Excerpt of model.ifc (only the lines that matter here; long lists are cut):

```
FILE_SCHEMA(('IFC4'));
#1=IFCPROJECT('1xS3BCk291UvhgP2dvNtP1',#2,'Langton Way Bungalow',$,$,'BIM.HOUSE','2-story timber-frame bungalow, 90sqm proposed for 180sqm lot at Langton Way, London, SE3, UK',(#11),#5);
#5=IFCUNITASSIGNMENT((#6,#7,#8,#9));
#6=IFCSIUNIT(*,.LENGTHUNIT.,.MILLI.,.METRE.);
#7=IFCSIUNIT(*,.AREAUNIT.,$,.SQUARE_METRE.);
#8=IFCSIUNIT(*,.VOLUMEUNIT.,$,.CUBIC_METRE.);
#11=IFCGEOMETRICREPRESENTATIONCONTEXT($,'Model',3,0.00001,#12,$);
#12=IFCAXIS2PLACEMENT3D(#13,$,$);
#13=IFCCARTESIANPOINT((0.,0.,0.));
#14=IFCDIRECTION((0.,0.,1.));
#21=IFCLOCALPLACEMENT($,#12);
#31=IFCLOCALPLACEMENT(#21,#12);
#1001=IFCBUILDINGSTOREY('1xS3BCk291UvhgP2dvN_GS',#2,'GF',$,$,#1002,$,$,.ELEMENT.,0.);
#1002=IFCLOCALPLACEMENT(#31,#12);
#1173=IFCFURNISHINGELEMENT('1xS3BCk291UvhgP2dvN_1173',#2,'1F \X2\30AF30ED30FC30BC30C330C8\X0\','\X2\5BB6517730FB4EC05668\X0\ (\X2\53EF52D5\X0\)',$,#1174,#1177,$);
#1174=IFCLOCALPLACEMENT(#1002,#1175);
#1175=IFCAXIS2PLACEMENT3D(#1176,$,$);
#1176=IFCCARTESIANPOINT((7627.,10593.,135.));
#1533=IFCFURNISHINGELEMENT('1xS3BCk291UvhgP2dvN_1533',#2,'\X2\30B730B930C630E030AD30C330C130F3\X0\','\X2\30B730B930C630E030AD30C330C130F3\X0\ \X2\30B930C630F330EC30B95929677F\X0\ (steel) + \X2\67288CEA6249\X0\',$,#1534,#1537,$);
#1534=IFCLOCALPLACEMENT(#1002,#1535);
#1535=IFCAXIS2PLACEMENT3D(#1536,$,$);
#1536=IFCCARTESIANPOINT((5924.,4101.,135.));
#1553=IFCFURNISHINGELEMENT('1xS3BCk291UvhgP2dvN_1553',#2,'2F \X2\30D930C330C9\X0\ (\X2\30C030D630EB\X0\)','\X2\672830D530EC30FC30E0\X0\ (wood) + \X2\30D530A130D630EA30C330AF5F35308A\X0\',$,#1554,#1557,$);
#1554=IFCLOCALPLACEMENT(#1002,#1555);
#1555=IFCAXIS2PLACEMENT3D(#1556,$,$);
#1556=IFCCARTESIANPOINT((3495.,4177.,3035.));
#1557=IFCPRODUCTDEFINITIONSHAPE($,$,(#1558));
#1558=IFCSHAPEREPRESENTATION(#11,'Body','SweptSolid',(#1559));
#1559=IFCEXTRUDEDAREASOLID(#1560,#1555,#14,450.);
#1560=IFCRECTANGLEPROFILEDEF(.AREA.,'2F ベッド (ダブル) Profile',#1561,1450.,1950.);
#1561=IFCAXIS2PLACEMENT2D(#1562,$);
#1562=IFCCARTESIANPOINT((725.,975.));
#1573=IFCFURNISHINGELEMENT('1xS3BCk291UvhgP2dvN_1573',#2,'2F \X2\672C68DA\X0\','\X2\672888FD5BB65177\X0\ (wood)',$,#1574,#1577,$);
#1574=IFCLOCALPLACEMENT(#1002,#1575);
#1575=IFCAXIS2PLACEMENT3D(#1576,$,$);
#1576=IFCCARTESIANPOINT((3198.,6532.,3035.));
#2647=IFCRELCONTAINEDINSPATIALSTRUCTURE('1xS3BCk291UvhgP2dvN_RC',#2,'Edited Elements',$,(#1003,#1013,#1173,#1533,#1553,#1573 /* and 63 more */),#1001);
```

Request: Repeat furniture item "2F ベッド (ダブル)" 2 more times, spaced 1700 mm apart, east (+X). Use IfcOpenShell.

```python
import numpy as np
import ifcopenshell
import ifcopenshell.api.geometry
import ifcopenshell.api.root
import ifcopenshell.util.element
import ifcopenshell.util.placement
import ifcopenshell.util.unit

model = ifcopenshell.open("model.ifc")
unit_scale = ifcopenshell.util.unit.calculate_unit_scale(model)


def reuse_history(source, copy):
    """copy_class also copies each property set's owner history, people and application; keep the originals."""
    for rel in copy.IsDefinedBy:
        if rel.is_a("IfcRelDefinesByProperties") and (history := rel.RelatingPropertyDefinition.OwnerHistory):
            rel.RelatingPropertyDefinition.OwnerHistory = source.OwnerHistory
            ifcopenshell.util.element.remove_deep2(model, history)


source = model.by_id(1553)
base = ifcopenshell.util.placement.get_local_placement(source.ObjectPlacement)
step = np.array([1.0, 0.0, 0.0]) * 1.7 / unit_scale

for i in range(1, 3):
    copy = ifcopenshell.api.root.copy_class(model, product=source)
    copy.Representation = ifcopenshell.util.element.copy_deep(
        model, source.Representation, exclude=["IfcGeometricRepresentationContext", "IfcRepresentationMap"]
    )
    reuse_history(source, copy)
    matrix = base.copy()
    matrix[:3, 3] += i * step
    print("added at", matrix[:3, 3].round(3) + 0.0)
    ifcopenshell.api.geometry.edit_object_placement(model, product=copy, matrix=matrix, is_si=False)

model.write("model_rev.ifc")
```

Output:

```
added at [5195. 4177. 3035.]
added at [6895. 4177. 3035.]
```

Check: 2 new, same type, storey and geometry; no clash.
